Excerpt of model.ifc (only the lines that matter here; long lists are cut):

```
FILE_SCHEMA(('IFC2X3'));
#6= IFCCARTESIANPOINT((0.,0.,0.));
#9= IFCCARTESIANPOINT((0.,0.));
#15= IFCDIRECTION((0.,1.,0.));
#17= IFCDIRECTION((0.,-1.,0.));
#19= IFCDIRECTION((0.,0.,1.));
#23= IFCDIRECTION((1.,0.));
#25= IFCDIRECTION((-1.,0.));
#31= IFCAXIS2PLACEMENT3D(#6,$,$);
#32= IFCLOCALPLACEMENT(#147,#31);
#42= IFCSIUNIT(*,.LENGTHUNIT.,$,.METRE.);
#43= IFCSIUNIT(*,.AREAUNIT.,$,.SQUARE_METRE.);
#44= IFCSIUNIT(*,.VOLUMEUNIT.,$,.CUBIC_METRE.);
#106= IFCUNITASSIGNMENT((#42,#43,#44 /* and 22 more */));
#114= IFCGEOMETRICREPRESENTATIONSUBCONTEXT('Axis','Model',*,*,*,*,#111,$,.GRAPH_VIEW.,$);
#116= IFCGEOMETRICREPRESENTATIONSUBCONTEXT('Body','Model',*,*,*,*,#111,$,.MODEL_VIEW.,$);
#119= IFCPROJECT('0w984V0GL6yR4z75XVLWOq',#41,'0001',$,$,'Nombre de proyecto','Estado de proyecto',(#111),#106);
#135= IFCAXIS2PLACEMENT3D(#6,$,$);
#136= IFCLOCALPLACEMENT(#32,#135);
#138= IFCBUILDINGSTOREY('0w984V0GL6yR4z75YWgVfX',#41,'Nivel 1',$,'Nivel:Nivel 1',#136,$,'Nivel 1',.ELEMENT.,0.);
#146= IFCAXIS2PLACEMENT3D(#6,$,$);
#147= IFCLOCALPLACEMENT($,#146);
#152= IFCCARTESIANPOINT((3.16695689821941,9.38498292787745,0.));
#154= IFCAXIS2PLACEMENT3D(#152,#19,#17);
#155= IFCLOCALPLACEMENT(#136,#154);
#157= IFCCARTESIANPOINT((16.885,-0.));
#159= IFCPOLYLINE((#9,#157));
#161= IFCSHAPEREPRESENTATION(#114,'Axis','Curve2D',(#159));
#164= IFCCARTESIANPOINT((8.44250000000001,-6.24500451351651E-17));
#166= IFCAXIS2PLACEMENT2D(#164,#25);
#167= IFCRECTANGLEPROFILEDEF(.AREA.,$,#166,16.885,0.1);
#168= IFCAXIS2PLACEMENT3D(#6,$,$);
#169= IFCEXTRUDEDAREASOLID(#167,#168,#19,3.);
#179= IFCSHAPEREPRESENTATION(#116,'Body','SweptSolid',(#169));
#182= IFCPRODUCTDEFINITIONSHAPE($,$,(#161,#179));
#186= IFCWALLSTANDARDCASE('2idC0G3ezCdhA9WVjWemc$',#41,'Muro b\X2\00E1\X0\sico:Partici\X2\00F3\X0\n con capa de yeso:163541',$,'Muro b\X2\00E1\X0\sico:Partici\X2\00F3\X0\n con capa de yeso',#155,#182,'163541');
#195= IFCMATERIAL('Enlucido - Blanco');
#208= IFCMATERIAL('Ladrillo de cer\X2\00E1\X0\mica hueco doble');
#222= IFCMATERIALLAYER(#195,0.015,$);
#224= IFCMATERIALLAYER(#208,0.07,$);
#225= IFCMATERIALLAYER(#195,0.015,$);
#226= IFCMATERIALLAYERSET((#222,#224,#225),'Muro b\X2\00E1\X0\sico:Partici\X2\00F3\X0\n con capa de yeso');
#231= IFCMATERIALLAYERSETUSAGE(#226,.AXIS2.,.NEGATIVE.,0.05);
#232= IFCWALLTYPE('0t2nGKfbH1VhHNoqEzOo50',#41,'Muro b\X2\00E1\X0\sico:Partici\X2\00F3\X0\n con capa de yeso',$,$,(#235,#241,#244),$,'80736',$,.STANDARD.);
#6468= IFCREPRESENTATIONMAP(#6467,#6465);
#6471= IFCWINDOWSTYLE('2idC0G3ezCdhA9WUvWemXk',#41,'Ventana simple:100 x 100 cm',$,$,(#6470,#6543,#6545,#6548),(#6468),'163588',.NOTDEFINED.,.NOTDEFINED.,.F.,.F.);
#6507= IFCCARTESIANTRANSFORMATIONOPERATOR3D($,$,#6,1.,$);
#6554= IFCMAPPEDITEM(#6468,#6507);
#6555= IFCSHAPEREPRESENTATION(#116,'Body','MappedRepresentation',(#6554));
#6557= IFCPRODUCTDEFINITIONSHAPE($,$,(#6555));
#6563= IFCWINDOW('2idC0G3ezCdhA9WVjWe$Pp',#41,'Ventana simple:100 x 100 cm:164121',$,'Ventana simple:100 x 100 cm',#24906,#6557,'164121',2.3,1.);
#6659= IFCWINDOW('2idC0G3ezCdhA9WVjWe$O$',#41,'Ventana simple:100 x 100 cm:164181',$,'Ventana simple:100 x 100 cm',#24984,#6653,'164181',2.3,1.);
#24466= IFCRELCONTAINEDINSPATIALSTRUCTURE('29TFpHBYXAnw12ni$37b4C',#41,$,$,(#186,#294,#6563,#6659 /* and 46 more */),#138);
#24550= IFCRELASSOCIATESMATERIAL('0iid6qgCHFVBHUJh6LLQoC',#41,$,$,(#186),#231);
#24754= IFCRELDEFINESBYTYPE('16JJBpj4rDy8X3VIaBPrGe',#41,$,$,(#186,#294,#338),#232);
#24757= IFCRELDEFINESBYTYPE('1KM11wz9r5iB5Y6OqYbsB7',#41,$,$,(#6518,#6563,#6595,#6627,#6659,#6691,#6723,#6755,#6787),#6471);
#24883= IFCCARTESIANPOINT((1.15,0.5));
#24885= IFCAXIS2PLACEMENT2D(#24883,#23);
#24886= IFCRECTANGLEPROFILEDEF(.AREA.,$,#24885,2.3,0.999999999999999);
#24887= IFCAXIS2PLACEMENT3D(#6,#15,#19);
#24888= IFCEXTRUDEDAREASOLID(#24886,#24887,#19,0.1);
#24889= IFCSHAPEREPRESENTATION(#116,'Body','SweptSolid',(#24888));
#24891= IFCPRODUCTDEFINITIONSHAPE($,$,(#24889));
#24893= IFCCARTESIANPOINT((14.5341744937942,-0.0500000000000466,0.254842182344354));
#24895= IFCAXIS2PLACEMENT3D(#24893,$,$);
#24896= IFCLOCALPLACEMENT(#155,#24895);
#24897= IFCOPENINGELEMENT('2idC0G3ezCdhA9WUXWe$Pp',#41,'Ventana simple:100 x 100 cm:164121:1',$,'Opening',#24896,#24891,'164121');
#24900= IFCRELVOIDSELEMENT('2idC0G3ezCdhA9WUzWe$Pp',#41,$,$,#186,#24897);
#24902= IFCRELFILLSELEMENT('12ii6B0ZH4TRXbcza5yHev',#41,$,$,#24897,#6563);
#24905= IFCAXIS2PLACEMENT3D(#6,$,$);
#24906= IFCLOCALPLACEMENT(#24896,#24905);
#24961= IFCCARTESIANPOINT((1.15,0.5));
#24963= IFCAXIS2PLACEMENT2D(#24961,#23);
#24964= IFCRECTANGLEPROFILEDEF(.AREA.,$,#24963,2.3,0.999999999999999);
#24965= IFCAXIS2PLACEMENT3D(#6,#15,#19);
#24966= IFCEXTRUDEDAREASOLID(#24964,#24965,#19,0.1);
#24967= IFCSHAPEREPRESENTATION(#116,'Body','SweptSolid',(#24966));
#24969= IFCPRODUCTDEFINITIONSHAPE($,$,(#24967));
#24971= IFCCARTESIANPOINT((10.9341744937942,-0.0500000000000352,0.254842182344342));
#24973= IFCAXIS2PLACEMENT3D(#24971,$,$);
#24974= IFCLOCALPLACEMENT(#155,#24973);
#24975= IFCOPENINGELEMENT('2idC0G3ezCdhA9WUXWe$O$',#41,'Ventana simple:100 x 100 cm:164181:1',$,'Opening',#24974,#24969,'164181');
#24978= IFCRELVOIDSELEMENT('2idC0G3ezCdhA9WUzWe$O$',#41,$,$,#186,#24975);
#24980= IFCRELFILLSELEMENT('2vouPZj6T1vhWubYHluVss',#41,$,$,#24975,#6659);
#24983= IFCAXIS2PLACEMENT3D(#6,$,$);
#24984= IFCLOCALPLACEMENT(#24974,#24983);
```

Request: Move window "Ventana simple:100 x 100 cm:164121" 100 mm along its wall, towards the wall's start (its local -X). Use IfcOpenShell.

```python
import ifcopenshell
import ifcopenshell.api.geometry
import ifcopenshell.util.placement

model = ifcopenshell.open("model.ifc")

window = model.by_id(6563)
opening = window.FillsVoids[0].RelatingOpeningElement
wall = opening.VoidsElements[0].RelatingBuildingElement

wall_matrix = ifcopenshell.util.placement.get_local_placement(wall.ObjectPlacement)
shift = wall_matrix[:3, 0] * -0.1
before = ifcopenshell.util.placement.get_local_placement(window.ObjectPlacement)[:3, 3].copy()

# The window is placed relative to its opening, so it follows when the opening moves.
matrix = ifcopenshell.util.placement.get_local_placement(opening.ObjectPlacement)
matrix[:3, 3] += shift
ifcopenshell.api.geometry.edit_object_placement(
    model, product=opening, matrix=matrix, is_si=False, should_transform_children=True
)

after = ifcopenshell.util.placement.get_local_placement(window.ObjectPlacement)[:3, 3]
print("window moved by", (after - before).round(3) + 0.0)

model.write("model_v2.ifc")
```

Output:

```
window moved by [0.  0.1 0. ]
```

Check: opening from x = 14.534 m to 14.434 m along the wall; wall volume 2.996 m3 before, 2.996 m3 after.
